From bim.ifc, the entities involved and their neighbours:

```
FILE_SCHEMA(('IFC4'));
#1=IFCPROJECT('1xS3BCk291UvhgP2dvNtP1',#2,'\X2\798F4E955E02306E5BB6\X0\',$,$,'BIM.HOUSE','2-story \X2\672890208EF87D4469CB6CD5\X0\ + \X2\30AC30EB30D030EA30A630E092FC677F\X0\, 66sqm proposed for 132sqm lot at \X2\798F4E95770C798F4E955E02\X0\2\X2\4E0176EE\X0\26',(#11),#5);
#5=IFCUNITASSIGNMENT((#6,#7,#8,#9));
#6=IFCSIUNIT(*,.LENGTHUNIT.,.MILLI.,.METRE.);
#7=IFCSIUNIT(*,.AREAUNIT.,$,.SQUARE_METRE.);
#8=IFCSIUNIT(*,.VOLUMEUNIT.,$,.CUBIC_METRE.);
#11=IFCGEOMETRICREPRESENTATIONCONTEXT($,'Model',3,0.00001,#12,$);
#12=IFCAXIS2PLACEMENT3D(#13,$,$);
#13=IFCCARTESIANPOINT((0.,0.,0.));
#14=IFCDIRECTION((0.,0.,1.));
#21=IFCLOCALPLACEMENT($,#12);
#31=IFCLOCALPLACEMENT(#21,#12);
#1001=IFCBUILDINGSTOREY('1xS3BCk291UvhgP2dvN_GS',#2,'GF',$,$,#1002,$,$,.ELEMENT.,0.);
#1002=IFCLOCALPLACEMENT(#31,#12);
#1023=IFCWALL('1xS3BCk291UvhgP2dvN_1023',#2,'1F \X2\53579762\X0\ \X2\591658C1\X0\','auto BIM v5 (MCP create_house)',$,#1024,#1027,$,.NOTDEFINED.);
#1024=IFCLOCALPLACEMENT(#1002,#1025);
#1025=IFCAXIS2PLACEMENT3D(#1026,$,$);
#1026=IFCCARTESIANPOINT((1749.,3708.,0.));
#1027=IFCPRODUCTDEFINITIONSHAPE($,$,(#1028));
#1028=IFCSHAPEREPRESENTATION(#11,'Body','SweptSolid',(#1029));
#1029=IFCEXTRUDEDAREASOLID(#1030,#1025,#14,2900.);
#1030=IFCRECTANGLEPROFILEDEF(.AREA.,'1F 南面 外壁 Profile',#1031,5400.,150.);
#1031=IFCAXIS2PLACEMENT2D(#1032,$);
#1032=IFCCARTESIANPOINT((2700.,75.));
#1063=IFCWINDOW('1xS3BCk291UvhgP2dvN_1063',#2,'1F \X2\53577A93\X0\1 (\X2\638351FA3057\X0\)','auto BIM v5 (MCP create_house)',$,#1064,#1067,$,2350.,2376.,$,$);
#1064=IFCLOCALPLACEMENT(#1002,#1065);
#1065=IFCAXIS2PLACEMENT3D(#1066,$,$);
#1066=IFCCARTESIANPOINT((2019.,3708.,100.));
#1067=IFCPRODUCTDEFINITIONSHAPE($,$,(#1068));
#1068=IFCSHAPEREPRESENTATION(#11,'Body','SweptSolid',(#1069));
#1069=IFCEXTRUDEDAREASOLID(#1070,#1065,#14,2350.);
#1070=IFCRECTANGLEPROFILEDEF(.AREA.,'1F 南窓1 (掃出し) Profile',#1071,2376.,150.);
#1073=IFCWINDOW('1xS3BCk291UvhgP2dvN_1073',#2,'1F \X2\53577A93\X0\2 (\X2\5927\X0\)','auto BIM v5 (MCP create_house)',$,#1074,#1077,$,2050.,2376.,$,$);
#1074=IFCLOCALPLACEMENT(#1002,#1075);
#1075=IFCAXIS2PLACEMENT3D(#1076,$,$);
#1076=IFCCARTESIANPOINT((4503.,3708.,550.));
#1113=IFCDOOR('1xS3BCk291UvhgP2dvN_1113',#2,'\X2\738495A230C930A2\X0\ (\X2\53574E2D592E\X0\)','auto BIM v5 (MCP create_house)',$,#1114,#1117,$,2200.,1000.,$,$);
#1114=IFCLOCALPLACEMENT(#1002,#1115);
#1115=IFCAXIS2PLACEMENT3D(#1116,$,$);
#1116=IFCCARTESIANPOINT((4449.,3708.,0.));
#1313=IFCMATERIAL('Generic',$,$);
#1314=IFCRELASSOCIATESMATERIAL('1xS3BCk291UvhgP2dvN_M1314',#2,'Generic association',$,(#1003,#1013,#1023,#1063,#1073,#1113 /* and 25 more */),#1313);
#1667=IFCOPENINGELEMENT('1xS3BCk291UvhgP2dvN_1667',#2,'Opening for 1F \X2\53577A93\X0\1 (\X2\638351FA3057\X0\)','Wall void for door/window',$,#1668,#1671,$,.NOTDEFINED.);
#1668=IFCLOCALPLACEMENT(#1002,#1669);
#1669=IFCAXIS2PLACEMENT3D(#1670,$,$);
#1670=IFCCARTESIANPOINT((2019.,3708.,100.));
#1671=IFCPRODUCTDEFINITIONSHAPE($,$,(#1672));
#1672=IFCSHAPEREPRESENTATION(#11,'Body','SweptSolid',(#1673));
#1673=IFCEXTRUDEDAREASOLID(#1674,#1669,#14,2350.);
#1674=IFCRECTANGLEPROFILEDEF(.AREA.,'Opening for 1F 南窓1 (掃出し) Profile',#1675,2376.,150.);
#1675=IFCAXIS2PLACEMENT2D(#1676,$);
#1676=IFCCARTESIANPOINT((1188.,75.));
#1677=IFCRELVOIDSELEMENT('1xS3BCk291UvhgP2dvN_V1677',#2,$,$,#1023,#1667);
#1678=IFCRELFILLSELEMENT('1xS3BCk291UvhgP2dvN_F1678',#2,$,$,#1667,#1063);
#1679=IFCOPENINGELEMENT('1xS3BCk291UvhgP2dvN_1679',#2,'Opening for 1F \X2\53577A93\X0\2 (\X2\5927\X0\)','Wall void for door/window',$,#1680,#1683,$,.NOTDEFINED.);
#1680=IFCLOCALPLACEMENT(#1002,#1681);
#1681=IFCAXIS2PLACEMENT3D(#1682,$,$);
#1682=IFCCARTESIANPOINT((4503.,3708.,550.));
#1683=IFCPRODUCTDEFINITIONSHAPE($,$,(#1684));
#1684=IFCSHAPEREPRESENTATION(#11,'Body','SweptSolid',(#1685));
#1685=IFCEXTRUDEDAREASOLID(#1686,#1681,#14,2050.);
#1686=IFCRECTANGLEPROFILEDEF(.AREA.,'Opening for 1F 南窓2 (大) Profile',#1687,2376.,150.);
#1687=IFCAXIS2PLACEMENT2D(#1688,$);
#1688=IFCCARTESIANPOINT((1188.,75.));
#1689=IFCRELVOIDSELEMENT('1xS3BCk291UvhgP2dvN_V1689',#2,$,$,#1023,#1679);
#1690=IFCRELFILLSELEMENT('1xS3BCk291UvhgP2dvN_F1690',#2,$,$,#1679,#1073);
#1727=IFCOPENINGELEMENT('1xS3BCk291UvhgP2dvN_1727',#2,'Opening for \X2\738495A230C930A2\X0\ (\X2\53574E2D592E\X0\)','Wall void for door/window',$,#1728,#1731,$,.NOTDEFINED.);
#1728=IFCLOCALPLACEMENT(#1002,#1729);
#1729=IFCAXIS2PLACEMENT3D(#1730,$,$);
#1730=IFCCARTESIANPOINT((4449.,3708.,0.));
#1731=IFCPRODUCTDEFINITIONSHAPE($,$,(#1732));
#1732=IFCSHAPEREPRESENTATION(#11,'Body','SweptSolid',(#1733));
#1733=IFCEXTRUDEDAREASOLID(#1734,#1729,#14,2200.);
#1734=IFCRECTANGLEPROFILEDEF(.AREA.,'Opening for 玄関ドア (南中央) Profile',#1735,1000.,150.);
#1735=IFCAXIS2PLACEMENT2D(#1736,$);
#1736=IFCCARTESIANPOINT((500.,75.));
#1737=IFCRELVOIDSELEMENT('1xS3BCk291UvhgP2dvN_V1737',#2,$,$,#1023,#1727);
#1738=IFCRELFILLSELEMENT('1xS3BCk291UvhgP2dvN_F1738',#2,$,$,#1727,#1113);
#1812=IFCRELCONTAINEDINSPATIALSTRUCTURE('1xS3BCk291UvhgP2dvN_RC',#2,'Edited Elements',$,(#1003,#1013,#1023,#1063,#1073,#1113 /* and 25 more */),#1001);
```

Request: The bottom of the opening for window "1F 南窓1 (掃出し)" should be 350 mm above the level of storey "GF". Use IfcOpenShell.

```python
import numpy as np
import ifcopenshell
import ifcopenshell.api.geometry
import ifcopenshell.geom
import ifcopenshell.util.element
import ifcopenshell.util.placement
import ifcopenshell.util.shape
import ifcopenshell.util.unit

model = ifcopenshell.open("bim.ifc")
unit_scale = ifcopenshell.util.unit.calculate_unit_scale(model)

window = model.by_guid("1xS3BCk291UvhgP2dvN_1063")
opening = window.FillsVoids[0].RelatingOpeningElement
storey = ifcopenshell.util.element.get_container(window, ifc_class="IfcBuildingStorey")
level = ifcopenshell.util.placement.get_local_placement(storey.ObjectPlacement)[2, 3]

# The opening's origin need not be at the sill, so measure its lowest point.
shape = ifcopenshell.geom.create_shape(ifcopenshell.geom.settings(), opening)
bottom = ifcopenshell.util.shape.get_shape_bottom_elevation(shape, shape.geometry) / unit_scale
dz = level + 0.35 / unit_scale - bottom

shift = np.array([0.0, 0.0, dz])
# The window is not placed relative to its opening, so move both.
for product in (opening, window):
    matrix = ifcopenshell.util.placement.get_local_placement(product.ObjectPlacement)
    matrix[:3, 3] += shift
    ifcopenshell.api.geometry.edit_object_placement(model, product=product, matrix=matrix, is_si=False)

print(f"moved by {dz * unit_scale:+.3f} m")

model.write("bim_updated.ifc")
```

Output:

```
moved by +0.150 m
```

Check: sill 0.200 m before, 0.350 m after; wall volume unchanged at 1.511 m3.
